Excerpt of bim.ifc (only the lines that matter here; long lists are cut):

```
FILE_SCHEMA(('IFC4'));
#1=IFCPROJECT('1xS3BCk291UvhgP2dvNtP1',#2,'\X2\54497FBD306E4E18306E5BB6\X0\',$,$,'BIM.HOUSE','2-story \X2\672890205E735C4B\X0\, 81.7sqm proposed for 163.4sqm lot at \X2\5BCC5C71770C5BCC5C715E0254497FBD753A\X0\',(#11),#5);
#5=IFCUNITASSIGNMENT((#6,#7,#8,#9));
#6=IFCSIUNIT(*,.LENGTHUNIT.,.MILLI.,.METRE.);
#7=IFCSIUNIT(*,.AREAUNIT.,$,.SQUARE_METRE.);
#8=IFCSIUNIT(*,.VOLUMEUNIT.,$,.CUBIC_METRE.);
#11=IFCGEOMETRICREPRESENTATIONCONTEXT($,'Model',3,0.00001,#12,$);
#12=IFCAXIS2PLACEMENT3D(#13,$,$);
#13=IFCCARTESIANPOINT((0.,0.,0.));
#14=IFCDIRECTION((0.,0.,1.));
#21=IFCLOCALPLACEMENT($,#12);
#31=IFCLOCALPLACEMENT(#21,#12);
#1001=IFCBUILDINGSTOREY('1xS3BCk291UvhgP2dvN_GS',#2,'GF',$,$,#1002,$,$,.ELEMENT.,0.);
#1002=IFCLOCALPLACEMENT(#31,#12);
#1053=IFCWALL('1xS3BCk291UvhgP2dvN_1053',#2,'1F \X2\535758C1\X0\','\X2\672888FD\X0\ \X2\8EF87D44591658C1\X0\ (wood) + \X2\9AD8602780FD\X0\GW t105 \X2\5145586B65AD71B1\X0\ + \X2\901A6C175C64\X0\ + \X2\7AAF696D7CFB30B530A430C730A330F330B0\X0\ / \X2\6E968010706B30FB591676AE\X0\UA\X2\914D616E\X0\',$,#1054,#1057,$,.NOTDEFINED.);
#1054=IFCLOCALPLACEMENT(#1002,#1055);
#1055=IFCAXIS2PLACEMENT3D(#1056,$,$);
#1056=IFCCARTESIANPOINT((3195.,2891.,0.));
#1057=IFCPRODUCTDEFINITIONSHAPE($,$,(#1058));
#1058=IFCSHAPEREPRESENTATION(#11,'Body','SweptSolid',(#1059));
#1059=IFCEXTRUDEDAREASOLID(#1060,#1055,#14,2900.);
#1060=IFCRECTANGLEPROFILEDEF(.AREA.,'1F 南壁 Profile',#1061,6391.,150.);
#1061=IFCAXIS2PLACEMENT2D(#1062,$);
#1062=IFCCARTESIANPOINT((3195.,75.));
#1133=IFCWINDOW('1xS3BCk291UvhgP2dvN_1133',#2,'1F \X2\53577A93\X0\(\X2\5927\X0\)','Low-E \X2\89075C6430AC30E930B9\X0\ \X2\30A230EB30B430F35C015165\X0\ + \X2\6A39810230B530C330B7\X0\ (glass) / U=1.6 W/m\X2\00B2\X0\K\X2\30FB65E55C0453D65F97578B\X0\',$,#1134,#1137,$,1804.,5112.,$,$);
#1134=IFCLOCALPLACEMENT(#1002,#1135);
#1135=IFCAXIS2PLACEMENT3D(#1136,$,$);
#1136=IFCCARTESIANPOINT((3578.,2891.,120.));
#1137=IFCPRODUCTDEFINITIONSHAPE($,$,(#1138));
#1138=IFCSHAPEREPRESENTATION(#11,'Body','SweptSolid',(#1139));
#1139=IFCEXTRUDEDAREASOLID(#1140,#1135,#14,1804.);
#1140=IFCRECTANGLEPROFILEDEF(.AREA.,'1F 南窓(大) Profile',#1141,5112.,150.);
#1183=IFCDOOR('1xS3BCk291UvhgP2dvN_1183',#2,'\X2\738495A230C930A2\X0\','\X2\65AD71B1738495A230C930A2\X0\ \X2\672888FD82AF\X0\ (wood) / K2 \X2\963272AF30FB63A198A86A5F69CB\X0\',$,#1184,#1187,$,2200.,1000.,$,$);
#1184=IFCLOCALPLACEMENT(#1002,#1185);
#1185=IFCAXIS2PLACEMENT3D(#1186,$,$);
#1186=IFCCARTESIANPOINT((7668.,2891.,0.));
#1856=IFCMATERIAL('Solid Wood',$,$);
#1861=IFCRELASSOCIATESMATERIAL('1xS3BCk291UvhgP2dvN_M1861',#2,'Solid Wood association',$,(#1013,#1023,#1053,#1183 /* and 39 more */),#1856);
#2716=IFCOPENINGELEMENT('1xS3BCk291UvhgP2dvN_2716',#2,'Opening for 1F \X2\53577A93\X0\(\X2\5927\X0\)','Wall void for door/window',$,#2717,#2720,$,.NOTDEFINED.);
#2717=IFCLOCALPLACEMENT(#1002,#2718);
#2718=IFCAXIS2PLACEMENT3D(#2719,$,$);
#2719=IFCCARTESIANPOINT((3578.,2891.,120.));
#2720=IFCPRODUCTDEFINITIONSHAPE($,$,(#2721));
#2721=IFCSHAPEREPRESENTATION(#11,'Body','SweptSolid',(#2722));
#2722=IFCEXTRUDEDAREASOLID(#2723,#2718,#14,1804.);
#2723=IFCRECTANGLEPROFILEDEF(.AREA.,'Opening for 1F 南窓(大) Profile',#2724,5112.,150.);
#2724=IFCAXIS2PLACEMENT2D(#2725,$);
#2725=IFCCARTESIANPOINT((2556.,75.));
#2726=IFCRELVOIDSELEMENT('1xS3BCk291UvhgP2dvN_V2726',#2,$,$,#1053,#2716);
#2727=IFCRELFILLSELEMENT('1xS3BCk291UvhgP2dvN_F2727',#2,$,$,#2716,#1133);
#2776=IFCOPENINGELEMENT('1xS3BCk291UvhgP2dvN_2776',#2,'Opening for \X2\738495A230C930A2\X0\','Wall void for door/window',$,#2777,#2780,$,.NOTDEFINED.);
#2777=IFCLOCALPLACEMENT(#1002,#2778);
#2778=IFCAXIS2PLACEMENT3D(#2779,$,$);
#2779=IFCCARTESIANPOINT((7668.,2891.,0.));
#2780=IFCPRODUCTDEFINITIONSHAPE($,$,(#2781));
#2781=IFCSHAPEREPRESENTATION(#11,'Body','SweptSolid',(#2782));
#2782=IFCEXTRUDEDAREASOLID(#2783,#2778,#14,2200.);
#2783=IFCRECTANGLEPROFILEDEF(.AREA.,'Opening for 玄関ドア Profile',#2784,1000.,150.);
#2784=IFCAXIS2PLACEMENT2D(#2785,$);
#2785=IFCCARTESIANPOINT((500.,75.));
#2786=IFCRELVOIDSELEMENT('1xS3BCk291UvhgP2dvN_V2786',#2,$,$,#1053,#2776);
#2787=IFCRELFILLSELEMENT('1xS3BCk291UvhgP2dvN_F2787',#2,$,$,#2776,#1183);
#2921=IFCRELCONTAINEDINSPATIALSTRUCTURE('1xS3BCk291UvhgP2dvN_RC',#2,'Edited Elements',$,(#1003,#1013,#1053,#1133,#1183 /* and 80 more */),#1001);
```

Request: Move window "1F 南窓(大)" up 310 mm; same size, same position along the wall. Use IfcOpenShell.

```python
import numpy as np
import ifcopenshell
import ifcopenshell.api.geometry
import ifcopenshell.util.placement
import ifcopenshell.util.unit

model = ifcopenshell.open("bim.ifc")
unit_scale = ifcopenshell.util.unit.calculate_unit_scale(model)

window = model.by_guid("1xS3BCk291UvhgP2dvN_1133")
opening = window.FillsVoids[0].RelatingOpeningElement
dz = 310.0

shift = np.array([0.0, 0.0, dz])
# The window is not placed relative to its opening, so move both.
for product in (opening, window):
    matrix = ifcopenshell.util.placement.get_local_placement(product.ObjectPlacement)
    matrix[:3, 3] += shift
    ifcopenshell.api.geometry.edit_object_placement(model, product=product, matrix=matrix, is_si=False)

print(f"moved by {dz * unit_scale:+.3f} m")

model.write("bim_v2.ifc")
```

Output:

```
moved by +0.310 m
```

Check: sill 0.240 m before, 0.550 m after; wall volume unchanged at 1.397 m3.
